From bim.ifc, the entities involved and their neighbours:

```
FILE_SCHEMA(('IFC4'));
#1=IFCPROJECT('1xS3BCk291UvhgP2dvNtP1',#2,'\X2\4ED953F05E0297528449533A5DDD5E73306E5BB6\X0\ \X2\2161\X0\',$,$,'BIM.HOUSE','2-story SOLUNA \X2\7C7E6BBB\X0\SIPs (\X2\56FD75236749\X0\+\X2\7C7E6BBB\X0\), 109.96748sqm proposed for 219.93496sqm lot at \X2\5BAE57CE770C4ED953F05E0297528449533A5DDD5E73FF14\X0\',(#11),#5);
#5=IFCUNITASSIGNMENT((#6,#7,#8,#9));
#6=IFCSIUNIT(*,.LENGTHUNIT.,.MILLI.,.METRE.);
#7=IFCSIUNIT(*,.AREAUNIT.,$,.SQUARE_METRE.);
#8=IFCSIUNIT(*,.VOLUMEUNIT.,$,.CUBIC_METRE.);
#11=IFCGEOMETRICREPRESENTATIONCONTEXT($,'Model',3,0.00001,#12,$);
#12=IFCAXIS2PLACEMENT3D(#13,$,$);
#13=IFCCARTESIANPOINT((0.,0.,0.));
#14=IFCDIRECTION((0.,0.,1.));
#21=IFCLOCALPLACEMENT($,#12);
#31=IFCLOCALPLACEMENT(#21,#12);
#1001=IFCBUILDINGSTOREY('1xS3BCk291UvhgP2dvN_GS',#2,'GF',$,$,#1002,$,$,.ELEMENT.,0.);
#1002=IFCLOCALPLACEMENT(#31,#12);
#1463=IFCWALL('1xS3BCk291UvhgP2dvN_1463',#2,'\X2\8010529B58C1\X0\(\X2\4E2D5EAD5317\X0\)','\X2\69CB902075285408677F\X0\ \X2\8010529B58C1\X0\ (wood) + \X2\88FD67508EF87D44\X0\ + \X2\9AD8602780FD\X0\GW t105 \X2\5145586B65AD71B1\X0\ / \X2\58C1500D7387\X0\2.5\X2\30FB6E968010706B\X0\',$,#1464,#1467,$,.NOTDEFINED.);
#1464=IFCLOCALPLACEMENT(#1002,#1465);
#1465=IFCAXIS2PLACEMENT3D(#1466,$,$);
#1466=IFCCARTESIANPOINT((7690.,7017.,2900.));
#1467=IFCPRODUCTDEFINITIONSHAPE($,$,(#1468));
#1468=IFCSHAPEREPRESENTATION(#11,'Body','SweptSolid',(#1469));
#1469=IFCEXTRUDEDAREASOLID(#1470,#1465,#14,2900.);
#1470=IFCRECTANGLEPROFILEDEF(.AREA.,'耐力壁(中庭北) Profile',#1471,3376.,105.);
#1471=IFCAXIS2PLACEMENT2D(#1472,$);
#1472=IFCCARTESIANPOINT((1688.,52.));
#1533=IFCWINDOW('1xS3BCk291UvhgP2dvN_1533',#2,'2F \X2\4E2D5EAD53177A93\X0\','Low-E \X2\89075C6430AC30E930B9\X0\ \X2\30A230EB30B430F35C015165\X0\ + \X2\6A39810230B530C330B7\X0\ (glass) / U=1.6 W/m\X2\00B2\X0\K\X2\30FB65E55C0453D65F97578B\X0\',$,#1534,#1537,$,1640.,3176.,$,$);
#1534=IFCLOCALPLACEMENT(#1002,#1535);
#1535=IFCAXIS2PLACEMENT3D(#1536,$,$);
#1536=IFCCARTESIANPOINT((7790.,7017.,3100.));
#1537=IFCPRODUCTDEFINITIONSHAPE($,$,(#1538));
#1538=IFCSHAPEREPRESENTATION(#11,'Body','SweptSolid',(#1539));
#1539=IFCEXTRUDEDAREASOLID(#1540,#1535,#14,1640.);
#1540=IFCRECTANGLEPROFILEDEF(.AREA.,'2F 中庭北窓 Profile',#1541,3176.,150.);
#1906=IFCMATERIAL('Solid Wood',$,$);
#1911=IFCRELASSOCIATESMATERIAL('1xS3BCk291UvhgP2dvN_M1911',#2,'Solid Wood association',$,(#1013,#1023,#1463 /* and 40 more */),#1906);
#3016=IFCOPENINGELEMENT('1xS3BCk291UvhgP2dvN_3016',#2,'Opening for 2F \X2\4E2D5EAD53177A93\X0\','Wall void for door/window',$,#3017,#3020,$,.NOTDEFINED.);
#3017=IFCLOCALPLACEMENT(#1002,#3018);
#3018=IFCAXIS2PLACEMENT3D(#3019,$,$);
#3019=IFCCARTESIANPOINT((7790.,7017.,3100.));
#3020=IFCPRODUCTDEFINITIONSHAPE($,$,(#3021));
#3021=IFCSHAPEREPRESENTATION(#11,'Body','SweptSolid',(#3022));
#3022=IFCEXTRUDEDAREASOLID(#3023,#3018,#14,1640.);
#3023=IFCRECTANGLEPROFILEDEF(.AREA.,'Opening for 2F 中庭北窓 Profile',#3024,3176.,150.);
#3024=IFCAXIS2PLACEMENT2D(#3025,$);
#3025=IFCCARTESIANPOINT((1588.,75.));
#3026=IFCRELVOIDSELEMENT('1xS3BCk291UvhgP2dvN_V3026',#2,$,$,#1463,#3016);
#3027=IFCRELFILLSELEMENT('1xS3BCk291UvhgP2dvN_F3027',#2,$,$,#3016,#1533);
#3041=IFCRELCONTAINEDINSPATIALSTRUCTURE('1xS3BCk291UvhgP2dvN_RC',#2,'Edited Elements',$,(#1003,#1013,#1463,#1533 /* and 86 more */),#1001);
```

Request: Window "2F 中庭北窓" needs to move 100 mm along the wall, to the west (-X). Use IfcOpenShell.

```python
import ifcopenshell
import ifcopenshell.api.geometry
import ifcopenshell.util.placement
import ifcopenshell.util.unit

model = ifcopenshell.open("bim.ifc")
unit_scale = ifcopenshell.util.unit.calculate_unit_scale(model)

window = model.by_guid("1xS3BCk291UvhgP2dvN_1533")
opening = window.FillsVoids[0].RelatingOpeningElement
wall = opening.VoidsElements[0].RelatingBuildingElement

wall_matrix = ifcopenshell.util.placement.get_local_placement(wall.ObjectPlacement)
shift = wall_matrix[:3, 0] * -0.1 / unit_scale
before = ifcopenshell.util.placement.get_local_placement(window.ObjectPlacement)[:3, 3].copy()

# The window is not placed relative to its opening, so move both.
for product in (opening, window):
    matrix = ifcopenshell.util.placement.get_local_placement(product.ObjectPlacement)
    matrix[:3, 3] += shift
    ifcopenshell.api.geometry.edit_object_placement(model, product=product, matrix=matrix, is_si=False)

after = ifcopenshell.util.placement.get_local_placement(window.ObjectPlacement)[:3, 3]
print("window moved by", (after - before).round(3) + 0.0)

model.write("bim-out.ifc")
```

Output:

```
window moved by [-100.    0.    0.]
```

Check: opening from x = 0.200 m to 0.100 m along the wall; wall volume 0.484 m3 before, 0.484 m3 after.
